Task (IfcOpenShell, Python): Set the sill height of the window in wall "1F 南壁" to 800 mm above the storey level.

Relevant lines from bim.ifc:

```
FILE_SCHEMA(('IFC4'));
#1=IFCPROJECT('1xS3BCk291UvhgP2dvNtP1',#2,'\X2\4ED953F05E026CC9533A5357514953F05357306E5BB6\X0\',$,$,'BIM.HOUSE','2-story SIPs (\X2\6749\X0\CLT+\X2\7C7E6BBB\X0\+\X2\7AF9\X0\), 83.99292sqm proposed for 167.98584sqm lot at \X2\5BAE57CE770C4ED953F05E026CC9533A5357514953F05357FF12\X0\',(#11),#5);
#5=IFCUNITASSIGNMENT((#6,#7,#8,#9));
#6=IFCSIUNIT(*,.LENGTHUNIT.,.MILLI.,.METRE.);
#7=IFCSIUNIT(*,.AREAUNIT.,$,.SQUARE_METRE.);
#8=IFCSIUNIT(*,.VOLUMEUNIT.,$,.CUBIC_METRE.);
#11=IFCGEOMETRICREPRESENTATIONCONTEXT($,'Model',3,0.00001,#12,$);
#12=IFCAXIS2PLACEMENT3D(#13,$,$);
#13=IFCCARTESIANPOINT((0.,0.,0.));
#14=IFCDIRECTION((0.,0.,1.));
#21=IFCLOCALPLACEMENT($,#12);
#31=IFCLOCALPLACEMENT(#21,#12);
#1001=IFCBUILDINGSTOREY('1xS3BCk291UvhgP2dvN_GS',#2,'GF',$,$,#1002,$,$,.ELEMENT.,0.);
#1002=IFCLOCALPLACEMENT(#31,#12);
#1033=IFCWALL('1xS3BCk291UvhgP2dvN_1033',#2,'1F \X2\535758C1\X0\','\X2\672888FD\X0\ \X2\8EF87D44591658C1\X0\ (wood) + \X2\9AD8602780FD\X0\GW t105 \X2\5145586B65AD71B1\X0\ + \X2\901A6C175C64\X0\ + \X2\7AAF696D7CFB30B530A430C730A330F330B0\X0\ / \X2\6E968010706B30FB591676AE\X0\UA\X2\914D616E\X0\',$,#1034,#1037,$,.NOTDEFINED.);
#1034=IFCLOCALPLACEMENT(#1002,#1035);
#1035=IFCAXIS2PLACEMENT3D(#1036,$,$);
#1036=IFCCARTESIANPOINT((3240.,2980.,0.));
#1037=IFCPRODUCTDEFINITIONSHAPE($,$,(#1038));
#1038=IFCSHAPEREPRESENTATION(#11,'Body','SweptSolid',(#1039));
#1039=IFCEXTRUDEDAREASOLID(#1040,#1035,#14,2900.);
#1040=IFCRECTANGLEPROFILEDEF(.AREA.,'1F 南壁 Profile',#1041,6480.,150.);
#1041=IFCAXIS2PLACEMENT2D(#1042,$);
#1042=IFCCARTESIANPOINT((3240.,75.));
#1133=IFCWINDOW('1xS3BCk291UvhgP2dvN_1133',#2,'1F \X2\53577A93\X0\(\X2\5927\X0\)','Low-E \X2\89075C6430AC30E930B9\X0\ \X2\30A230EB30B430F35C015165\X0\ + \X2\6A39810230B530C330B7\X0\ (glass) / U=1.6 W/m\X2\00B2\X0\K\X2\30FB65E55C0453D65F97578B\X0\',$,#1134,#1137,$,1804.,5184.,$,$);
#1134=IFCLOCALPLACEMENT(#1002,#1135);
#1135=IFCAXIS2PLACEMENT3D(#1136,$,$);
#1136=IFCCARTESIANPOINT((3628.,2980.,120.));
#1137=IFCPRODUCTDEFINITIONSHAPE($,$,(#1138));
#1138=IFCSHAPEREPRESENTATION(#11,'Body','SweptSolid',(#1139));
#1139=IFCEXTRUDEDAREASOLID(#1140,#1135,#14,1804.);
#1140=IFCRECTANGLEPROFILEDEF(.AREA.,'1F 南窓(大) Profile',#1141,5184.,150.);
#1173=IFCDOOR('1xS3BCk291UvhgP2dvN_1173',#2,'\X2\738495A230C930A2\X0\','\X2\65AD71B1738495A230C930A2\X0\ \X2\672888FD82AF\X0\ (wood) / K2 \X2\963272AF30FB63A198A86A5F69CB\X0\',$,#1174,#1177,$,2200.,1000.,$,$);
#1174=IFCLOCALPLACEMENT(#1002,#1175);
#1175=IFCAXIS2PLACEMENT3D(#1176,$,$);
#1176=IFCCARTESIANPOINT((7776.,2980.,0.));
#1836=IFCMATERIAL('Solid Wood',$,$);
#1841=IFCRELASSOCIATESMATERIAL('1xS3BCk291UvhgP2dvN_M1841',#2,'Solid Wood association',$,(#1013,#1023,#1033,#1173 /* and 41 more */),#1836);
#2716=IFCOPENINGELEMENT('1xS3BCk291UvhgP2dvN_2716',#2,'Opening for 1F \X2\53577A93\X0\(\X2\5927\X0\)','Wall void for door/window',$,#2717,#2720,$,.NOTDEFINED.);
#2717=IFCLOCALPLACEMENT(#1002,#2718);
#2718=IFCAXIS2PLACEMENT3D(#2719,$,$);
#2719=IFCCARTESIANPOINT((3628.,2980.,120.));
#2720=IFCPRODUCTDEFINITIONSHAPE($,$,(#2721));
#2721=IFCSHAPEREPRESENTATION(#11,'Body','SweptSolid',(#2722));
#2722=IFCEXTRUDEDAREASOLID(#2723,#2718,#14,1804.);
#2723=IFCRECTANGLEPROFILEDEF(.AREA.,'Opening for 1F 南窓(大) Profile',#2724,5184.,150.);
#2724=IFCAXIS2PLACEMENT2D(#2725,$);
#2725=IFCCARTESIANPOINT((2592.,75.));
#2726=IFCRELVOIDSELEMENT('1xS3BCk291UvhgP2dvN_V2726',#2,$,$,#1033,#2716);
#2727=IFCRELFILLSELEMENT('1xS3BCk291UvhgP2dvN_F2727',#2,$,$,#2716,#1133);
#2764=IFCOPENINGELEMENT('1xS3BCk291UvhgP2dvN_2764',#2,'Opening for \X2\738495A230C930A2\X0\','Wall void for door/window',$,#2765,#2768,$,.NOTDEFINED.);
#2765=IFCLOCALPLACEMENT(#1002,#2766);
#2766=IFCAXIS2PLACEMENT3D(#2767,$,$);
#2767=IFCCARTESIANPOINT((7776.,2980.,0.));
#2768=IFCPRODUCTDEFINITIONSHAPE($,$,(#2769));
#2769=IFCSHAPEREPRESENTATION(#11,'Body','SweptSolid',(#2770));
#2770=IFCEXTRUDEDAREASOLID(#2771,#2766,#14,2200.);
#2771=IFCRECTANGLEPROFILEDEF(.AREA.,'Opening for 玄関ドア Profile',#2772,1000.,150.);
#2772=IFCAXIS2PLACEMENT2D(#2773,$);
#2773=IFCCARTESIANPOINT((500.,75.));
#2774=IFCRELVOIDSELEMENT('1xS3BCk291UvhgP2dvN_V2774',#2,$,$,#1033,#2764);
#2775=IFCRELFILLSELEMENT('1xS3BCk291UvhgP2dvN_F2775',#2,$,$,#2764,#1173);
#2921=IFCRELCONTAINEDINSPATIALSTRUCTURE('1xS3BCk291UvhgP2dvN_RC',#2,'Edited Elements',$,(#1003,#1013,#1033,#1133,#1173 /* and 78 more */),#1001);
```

```python
import numpy as np
import ifcopenshell
import ifcopenshell.api.geometry
import ifcopenshell.geom
import ifcopenshell.util.element
import ifcopenshell.util.placement
import ifcopenshell.util.shape
import ifcopenshell.util.unit

model = ifcopenshell.open("bim.ifc")
unit_scale = ifcopenshell.util.unit.calculate_unit_scale(model)

window = model.by_guid("1xS3BCk291UvhgP2dvN_1133")
opening = window.FillsVoids[0].RelatingOpeningElement
storey = ifcopenshell.util.element.get_container(window, ifc_class="IfcBuildingStorey")
level = ifcopenshell.util.placement.get_local_placement(storey.ObjectPlacement)[2, 3]

# The opening's origin need not be at the sill, so measure its lowest point.
shape = ifcopenshell.geom.create_shape(ifcopenshell.geom.settings(), opening)
bottom = ifcopenshell.util.shape.get_shape_bottom_elevation(shape, shape.geometry) / unit_scale
dz = level + 800.0 - bottom

shift = np.array([0.0, 0.0, dz])
# The window is not placed relative to its opening, so move both.
for product in (opening, window):
    matrix = ifcopenshell.util.placement.get_local_placement(product.ObjectPlacement)
    matrix[:3, 3] += shift
    ifcopenshell.api.geometry.edit_object_placement(model, product=product, matrix=matrix, is_si=False)

print(f"moved by {dz * unit_scale:+.3f} m")

model.write("bim-out.ifc")
```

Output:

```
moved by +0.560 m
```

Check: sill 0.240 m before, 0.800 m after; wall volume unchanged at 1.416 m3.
